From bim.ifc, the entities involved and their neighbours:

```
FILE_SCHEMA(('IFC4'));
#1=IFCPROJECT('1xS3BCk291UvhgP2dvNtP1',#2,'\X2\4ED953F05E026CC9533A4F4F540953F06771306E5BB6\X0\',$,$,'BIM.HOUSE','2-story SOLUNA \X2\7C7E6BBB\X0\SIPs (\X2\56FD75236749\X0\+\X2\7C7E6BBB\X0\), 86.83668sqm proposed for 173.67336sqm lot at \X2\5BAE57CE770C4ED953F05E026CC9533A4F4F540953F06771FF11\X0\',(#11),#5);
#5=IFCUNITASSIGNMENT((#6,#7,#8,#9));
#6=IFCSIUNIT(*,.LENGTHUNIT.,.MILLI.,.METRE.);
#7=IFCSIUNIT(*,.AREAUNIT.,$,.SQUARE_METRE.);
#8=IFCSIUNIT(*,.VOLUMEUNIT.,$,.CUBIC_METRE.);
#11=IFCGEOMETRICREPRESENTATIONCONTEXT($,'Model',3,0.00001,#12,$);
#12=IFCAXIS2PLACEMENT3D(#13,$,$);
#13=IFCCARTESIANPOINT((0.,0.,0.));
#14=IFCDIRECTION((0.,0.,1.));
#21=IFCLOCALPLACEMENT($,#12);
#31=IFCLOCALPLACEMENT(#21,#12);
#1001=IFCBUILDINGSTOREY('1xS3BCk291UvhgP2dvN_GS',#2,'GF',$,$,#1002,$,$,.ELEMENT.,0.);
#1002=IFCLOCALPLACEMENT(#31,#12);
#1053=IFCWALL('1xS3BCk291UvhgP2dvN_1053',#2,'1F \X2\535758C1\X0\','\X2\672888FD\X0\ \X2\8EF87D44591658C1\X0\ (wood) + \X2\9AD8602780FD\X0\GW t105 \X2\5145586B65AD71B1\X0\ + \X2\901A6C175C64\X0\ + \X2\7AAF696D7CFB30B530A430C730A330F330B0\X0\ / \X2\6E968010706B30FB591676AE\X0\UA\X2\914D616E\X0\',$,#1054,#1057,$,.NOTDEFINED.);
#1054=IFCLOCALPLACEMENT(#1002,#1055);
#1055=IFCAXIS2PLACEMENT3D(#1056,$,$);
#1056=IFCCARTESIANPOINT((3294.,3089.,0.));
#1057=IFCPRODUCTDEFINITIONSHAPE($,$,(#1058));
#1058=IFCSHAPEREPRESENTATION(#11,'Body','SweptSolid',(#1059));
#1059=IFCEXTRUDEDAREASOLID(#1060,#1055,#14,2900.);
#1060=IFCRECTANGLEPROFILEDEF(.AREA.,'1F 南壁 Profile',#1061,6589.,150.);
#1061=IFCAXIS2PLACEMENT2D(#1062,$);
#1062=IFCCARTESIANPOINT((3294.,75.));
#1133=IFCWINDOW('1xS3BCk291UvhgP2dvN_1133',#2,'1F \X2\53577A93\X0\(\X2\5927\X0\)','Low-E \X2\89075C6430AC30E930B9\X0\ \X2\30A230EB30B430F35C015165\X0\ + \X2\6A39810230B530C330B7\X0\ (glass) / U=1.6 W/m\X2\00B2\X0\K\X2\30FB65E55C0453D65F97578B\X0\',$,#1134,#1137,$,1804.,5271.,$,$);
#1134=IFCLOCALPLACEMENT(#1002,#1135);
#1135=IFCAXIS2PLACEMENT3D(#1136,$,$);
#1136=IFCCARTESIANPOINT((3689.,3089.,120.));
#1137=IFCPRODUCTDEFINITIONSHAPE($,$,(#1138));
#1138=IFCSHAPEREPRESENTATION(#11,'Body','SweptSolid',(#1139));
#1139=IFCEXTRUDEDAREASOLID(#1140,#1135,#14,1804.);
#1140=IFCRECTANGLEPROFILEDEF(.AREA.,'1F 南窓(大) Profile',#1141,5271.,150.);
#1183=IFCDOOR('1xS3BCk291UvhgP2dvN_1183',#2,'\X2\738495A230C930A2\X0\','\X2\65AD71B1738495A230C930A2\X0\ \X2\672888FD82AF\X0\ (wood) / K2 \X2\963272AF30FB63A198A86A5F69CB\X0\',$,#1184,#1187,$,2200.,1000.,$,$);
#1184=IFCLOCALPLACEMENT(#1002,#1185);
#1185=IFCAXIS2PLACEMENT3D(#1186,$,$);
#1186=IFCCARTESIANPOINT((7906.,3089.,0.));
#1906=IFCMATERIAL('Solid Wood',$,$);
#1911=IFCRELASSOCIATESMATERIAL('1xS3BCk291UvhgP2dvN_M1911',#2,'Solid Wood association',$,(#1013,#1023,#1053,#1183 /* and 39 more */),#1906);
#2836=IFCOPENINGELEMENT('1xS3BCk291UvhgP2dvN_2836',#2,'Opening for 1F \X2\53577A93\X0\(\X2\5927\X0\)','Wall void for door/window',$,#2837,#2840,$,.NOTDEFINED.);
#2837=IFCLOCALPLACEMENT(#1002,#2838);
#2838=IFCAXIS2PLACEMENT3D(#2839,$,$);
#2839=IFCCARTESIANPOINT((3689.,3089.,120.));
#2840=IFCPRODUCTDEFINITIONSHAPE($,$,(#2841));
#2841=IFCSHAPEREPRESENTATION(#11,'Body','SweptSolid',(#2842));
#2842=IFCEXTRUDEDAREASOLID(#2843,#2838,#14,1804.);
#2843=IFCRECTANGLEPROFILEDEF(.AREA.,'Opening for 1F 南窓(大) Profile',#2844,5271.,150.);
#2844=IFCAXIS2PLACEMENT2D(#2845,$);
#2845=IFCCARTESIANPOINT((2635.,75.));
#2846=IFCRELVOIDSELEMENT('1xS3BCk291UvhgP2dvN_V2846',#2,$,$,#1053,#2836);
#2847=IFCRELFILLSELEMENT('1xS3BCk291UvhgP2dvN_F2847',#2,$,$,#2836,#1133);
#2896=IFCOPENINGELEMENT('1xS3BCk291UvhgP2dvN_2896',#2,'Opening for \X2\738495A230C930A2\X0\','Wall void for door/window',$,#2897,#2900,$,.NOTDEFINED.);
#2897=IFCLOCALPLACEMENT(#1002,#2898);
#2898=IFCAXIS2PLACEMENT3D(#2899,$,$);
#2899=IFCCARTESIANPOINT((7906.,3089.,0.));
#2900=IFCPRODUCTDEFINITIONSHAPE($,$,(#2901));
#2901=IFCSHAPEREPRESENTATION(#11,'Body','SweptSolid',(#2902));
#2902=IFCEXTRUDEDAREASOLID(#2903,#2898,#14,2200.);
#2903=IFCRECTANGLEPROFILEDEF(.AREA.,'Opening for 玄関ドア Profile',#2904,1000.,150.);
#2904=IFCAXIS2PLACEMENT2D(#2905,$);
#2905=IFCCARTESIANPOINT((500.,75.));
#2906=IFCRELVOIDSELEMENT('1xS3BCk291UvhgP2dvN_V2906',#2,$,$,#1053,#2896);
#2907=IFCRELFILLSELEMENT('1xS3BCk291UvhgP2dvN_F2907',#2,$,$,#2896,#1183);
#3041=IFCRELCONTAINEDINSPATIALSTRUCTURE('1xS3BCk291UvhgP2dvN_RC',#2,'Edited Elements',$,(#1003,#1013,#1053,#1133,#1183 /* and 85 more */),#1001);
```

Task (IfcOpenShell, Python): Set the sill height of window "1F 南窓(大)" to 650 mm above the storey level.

```python
import numpy as np
import ifcopenshell
import ifcopenshell.api.geometry
import ifcopenshell.geom
import ifcopenshell.util.element
import ifcopenshell.util.placement
import ifcopenshell.util.shape
import ifcopenshell.util.unit

model = ifcopenshell.open("bim.ifc")
unit_scale = ifcopenshell.util.unit.calculate_unit_scale(model)

window = model.by_id(1133)
opening = window.FillsVoids[0].RelatingOpeningElement
storey = ifcopenshell.util.element.get_container(window, ifc_class="IfcBuildingStorey")
level = ifcopenshell.util.placement.get_local_placement(storey.ObjectPlacement)[2, 3]

# The opening's origin need not be at the sill, so measure its lowest point.
shape = ifcopenshell.geom.create_shape(ifcopenshell.geom.settings(), opening)
bottom = ifcopenshell.util.shape.get_shape_bottom_elevation(shape, shape.geometry) / unit_scale
dz = level + 0.65 / unit_scale - bottom

shift = np.array([0.0, 0.0, dz])
# The window is not placed relative to its opening, so move both.
for product in (opening, window):
    matrix = ifcopenshell.util.placement.get_local_placement(product.ObjectPlacement)
    matrix[:3, 3] += shift
    ifcopenshell.api.geometry.edit_object_placement(model, product=product, matrix=matrix, is_si=False)

print(f"moved by {dz * unit_scale:+.3f} m")

model.write("bim-out.ifc")
```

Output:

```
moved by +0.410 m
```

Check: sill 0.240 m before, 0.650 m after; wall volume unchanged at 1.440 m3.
